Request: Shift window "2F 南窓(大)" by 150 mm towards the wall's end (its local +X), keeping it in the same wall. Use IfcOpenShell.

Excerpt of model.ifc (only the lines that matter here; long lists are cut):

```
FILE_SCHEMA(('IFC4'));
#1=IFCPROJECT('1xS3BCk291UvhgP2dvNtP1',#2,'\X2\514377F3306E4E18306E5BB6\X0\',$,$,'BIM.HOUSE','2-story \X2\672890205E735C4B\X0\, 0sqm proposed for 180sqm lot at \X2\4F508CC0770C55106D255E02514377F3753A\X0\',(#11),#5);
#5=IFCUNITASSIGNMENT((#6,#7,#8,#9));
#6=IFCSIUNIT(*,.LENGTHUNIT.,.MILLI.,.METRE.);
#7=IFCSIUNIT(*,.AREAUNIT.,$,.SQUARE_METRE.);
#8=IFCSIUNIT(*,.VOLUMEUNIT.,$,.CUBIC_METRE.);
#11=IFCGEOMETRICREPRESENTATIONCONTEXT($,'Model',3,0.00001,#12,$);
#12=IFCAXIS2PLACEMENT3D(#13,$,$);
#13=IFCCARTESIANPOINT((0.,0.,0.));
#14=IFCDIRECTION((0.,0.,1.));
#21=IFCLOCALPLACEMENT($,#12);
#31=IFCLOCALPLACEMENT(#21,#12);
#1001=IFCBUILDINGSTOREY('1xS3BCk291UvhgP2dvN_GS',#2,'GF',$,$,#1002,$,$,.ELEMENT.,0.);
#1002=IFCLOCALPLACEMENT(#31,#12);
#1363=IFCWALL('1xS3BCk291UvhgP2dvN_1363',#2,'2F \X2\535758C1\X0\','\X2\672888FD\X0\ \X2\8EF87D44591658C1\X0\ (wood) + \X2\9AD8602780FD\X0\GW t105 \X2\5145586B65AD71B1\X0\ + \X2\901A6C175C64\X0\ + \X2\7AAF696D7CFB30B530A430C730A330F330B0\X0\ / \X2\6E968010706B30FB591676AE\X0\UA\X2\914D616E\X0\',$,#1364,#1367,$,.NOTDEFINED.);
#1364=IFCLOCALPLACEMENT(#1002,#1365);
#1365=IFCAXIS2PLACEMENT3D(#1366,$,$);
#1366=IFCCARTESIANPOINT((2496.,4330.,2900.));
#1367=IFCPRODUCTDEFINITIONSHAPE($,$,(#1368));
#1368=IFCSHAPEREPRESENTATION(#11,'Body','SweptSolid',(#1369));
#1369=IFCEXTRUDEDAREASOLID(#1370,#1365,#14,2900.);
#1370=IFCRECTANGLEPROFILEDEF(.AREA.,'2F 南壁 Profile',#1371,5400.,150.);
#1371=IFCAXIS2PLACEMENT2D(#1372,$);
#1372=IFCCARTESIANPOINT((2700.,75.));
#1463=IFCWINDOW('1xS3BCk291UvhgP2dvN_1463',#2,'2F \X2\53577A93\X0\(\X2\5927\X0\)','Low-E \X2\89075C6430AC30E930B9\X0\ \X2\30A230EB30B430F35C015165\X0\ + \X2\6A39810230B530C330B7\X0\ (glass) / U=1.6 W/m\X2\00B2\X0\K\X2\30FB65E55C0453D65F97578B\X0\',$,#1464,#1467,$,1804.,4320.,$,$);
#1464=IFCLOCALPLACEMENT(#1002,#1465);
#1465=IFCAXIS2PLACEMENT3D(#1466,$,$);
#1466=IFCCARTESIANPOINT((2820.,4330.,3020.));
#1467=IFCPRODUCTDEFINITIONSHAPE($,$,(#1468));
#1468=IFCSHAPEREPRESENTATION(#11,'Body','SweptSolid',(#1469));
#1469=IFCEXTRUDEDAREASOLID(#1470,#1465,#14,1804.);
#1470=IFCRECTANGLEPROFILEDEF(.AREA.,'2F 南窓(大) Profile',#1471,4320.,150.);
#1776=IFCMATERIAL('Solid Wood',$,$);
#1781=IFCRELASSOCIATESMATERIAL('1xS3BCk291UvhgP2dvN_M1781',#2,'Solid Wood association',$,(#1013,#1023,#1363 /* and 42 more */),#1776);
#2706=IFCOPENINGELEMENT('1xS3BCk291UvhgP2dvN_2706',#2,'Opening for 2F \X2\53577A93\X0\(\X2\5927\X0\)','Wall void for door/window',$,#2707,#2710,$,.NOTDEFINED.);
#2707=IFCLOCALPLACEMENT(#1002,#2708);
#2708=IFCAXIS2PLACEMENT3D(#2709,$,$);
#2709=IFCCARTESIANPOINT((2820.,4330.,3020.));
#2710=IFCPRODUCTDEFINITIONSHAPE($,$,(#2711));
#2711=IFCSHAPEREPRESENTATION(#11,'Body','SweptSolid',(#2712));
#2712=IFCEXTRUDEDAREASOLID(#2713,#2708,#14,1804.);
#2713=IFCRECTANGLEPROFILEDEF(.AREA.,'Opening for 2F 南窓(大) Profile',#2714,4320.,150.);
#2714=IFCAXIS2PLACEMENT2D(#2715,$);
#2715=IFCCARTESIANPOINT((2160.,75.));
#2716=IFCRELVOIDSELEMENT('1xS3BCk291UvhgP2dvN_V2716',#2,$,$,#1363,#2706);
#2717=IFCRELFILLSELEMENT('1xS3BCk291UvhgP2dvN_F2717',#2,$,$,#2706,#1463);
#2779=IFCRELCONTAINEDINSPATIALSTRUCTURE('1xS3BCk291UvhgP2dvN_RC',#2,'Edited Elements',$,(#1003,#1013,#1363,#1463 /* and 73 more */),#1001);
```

```python
import ifcopenshell
import ifcopenshell.api.geometry
import ifcopenshell.util.placement

model = ifcopenshell.open("model.ifc")

window = model.by_guid("1xS3BCk291UvhgP2dvN_1463")
opening = window.FillsVoids[0].RelatingOpeningElement
wall = opening.VoidsElements[0].RelatingBuildingElement

wall_matrix = ifcopenshell.util.placement.get_local_placement(wall.ObjectPlacement)
shift = wall_matrix[:3, 0] * 150.0
before = ifcopenshell.util.placement.get_local_placement(window.ObjectPlacement)[:3, 3].copy()

# The window is not placed relative to its opening, so move both.
for product in (opening, window):
    matrix = ifcopenshell.util.placement.get_local_placement(product.ObjectPlacement)
    matrix[:3, 3] += shift
    ifcopenshell.api.geometry.edit_object_placement(model, product=product, matrix=matrix, is_si=False)

after = ifcopenshell.util.placement.get_local_placement(window.ObjectPlacement)[:3, 3]
print("window moved by", (after - before).round(3) + 0.0)

model.write("model_v2.ifc")
```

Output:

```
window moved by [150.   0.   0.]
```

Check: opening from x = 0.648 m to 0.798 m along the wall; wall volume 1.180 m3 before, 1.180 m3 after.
